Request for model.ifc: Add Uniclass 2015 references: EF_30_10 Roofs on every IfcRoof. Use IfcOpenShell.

First a look at what the model holds.

```python
import ifcopenshell

model = ifcopenshell.open("model.ifc")
print(model.schema)
print("classifications:", [c.Name for c in model.by_type("IfcClassification")])
for ifc_class in ("IfcDoor", "IfcRoof", "IfcStair", "IfcWall", "IfcWindow"):
    print(ifc_class, len(model.by_type(ifc_class)))
```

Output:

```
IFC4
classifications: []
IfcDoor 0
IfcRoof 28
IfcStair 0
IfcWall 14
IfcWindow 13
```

```python
import ifcopenshell
import ifcopenshell.api.classification

model = ifcopenshell.open("model.ifc")

system = ifcopenshell.api.classification.add_classification(model, classification="Uniclass 2015")

codes = {
    "IfcRoof": ("EF_30_10", "Roofs"),
}
for ifc_class, (code, name) in codes.items():
    products = model.by_type(ifc_class)
    ifcopenshell.api.classification.add_reference(
        model, products=products, classification=system, identification=code, name=name
    )
    print(code, len(products))

model.write("model_v2.ifc")
```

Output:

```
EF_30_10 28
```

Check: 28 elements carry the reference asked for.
